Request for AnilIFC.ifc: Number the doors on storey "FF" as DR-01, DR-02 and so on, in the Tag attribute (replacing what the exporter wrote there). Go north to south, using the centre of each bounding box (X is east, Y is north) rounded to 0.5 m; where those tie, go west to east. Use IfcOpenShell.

First a look at what the model holds.

```python
import ifcopenshell
import ifcopenshell.util.element
import ifcopenshell.util.placement

model = ifcopenshell.open("AnilIFC.ifc")
print(model.schema)
storey = next(s for s in model.by_type("IfcBuildingStorey") if s.Name == "FF")
doors = [e for e in ifcopenshell.util.element.get_decomposition(storey) if e.is_a("IfcDoor")]
for e in sorted(doors, key=lambda e: e.id()):
    origin = ifcopenshell.util.placement.get_local_placement(e.ObjectPlacement)[:3, 3]
    print(e.id(), e.Tag, e.Name, origin.round(2) + 0.0, sep=" | ")
```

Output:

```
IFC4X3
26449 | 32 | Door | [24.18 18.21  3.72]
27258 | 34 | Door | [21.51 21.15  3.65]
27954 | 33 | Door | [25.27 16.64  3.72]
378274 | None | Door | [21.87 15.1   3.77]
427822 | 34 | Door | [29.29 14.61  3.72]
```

```python
import ifcopenshell
import ifcopenshell.geom
import ifcopenshell.util.element
import ifcopenshell.util.shape

model = ifcopenshell.open("AnilIFC.ifc")
settings = ifcopenshell.geom.settings()
settings.set("use-world-coords", True)


def centre(element):
    shape = ifcopenshell.geom.create_shape(settings, element)
    return ifcopenshell.util.shape.get_bbox_centroid(shape.geometry)


storey = next(s for s in model.by_type("IfcBuildingStorey") if s.Name == "FF")
doors = [e for e in ifcopenshell.util.element.get_decomposition(storey) if e.is_a("IfcDoor")]

# Insertion points can sit at a corner or the storey origin, so sort by the geometry (in metres).
centres = {e: centre(e) for e in doors}
doors.sort(key=lambda e: (-round(centres[e][1] / 0.5), centres[e][0]))

for i, e in enumerate(doors, start=1):
    number = f"DR-{i:02d}"
    e.Tag = number
    print(e.id(), number)

model.write("AnilIFC_v2.ifc")
```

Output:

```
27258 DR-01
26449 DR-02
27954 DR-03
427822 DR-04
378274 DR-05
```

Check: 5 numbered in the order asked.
